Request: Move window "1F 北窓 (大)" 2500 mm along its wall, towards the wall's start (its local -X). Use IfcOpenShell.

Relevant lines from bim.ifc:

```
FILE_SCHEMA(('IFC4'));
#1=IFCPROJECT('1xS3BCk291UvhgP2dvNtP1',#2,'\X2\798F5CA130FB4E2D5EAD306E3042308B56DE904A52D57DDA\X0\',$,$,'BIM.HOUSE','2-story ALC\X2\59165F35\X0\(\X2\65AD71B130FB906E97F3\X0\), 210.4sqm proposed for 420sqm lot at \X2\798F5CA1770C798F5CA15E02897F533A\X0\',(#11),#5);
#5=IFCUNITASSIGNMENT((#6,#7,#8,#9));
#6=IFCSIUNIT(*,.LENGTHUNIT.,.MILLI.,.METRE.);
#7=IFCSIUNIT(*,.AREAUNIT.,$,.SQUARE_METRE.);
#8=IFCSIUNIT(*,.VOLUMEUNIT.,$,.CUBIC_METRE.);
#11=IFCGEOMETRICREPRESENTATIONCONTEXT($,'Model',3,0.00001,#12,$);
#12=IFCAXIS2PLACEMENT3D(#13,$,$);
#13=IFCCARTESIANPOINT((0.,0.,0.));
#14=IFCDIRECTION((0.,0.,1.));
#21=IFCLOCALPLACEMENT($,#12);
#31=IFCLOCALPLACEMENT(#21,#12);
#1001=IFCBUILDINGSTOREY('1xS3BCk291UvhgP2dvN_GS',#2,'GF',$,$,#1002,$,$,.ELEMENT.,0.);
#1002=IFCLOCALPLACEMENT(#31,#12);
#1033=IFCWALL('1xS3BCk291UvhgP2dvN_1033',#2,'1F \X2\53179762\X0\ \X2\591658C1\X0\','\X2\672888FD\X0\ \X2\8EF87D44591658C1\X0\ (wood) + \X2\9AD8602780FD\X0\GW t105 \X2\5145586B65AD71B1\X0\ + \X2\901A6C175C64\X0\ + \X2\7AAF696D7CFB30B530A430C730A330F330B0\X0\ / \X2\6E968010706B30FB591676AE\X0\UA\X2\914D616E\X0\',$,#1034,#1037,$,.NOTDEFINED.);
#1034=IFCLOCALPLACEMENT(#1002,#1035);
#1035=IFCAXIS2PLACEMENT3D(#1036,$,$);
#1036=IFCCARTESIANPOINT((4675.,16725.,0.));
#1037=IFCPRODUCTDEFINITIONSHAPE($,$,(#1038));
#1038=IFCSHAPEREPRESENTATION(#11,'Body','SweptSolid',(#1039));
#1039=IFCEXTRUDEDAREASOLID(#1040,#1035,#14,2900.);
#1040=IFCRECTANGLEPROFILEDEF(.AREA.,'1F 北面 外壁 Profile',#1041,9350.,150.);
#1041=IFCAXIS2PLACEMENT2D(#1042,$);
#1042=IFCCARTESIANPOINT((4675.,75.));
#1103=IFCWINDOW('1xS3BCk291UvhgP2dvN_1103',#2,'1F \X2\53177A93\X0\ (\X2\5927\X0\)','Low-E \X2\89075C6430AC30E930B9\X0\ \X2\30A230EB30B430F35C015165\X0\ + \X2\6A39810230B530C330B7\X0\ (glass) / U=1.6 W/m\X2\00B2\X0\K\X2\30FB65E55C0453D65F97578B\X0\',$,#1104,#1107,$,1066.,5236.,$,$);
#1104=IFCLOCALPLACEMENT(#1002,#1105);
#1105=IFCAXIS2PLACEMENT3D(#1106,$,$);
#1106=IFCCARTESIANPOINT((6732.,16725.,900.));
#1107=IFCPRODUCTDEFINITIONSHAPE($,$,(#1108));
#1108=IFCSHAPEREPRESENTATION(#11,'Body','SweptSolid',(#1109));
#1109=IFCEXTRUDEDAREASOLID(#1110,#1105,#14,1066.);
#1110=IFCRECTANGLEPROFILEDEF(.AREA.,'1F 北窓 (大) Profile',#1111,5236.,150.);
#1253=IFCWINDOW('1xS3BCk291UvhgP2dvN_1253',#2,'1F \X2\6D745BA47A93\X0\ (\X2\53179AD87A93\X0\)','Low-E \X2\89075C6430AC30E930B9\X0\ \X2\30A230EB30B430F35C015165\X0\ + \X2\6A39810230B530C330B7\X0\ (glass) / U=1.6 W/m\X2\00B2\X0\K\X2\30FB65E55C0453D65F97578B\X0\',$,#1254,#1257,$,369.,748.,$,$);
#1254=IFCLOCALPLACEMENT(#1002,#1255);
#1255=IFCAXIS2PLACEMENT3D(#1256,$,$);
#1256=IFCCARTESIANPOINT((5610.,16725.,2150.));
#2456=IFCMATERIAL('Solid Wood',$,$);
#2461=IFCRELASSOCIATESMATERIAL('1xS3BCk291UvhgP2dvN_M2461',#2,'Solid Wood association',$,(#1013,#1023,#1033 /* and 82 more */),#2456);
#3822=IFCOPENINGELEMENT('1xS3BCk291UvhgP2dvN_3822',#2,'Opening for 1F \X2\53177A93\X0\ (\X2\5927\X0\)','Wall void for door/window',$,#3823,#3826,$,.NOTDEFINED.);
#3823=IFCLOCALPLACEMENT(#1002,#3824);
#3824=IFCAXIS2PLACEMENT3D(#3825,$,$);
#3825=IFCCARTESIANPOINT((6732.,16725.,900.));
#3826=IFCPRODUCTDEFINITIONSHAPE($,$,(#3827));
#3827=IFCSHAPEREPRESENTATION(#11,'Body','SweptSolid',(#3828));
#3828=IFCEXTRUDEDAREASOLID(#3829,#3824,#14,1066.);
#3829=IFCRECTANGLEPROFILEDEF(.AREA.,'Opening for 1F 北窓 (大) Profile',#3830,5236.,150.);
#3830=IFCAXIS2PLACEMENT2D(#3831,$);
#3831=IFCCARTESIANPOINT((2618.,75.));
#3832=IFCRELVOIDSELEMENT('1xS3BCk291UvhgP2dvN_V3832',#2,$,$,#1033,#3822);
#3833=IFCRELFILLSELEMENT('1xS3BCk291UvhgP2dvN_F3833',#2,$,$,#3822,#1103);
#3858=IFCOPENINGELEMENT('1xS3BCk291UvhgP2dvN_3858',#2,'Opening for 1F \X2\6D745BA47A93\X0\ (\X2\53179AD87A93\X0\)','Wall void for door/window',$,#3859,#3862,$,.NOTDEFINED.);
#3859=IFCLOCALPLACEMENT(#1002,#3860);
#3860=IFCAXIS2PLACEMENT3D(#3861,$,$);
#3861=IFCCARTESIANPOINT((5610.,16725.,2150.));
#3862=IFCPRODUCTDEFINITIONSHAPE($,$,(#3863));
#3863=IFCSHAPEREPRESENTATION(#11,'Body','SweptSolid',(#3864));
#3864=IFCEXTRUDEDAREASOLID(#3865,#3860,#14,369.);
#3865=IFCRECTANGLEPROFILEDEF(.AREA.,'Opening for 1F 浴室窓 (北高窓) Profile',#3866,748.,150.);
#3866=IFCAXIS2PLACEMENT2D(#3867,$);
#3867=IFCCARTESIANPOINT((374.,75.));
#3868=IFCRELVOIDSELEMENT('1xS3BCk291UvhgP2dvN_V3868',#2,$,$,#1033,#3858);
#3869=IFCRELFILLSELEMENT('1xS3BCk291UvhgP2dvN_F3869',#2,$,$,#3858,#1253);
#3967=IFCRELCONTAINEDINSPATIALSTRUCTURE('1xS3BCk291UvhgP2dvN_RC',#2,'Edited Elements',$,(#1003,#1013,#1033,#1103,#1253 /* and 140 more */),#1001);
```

```python
import ifcopenshell
import ifcopenshell.api.geometry
import ifcopenshell.util.placement
import ifcopenshell.util.unit

model = ifcopenshell.open("bim.ifc")
unit_scale = ifcopenshell.util.unit.calculate_unit_scale(model)

window = model.by_guid("1xS3BCk291UvhgP2dvN_1103")
opening = window.FillsVoids[0].RelatingOpeningElement
wall = opening.VoidsElements[0].RelatingBuildingElement

wall_matrix = ifcopenshell.util.placement.get_local_placement(wall.ObjectPlacement)
shift = wall_matrix[:3, 0] * -2.5 / unit_scale
before = ifcopenshell.util.placement.get_local_placement(window.ObjectPlacement)[:3, 3].copy()

# The window is not placed relative to its opening, so move both.
for product in (opening, window):
    matrix = ifcopenshell.util.placement.get_local_placement(product.ObjectPlacement)
    matrix[:3, 3] += shift
    ifcopenshell.api.geometry.edit_object_placement(model, product=product, matrix=matrix, is_si=False)

after = ifcopenshell.util.placement.get_local_placement(window.ObjectPlacement)[:3, 3]
print("window moved by", (after - before).round(3) + 0.0)

model.write("bim_edited.ifc")
```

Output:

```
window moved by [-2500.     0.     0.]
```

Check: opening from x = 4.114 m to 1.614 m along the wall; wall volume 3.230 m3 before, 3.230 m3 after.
